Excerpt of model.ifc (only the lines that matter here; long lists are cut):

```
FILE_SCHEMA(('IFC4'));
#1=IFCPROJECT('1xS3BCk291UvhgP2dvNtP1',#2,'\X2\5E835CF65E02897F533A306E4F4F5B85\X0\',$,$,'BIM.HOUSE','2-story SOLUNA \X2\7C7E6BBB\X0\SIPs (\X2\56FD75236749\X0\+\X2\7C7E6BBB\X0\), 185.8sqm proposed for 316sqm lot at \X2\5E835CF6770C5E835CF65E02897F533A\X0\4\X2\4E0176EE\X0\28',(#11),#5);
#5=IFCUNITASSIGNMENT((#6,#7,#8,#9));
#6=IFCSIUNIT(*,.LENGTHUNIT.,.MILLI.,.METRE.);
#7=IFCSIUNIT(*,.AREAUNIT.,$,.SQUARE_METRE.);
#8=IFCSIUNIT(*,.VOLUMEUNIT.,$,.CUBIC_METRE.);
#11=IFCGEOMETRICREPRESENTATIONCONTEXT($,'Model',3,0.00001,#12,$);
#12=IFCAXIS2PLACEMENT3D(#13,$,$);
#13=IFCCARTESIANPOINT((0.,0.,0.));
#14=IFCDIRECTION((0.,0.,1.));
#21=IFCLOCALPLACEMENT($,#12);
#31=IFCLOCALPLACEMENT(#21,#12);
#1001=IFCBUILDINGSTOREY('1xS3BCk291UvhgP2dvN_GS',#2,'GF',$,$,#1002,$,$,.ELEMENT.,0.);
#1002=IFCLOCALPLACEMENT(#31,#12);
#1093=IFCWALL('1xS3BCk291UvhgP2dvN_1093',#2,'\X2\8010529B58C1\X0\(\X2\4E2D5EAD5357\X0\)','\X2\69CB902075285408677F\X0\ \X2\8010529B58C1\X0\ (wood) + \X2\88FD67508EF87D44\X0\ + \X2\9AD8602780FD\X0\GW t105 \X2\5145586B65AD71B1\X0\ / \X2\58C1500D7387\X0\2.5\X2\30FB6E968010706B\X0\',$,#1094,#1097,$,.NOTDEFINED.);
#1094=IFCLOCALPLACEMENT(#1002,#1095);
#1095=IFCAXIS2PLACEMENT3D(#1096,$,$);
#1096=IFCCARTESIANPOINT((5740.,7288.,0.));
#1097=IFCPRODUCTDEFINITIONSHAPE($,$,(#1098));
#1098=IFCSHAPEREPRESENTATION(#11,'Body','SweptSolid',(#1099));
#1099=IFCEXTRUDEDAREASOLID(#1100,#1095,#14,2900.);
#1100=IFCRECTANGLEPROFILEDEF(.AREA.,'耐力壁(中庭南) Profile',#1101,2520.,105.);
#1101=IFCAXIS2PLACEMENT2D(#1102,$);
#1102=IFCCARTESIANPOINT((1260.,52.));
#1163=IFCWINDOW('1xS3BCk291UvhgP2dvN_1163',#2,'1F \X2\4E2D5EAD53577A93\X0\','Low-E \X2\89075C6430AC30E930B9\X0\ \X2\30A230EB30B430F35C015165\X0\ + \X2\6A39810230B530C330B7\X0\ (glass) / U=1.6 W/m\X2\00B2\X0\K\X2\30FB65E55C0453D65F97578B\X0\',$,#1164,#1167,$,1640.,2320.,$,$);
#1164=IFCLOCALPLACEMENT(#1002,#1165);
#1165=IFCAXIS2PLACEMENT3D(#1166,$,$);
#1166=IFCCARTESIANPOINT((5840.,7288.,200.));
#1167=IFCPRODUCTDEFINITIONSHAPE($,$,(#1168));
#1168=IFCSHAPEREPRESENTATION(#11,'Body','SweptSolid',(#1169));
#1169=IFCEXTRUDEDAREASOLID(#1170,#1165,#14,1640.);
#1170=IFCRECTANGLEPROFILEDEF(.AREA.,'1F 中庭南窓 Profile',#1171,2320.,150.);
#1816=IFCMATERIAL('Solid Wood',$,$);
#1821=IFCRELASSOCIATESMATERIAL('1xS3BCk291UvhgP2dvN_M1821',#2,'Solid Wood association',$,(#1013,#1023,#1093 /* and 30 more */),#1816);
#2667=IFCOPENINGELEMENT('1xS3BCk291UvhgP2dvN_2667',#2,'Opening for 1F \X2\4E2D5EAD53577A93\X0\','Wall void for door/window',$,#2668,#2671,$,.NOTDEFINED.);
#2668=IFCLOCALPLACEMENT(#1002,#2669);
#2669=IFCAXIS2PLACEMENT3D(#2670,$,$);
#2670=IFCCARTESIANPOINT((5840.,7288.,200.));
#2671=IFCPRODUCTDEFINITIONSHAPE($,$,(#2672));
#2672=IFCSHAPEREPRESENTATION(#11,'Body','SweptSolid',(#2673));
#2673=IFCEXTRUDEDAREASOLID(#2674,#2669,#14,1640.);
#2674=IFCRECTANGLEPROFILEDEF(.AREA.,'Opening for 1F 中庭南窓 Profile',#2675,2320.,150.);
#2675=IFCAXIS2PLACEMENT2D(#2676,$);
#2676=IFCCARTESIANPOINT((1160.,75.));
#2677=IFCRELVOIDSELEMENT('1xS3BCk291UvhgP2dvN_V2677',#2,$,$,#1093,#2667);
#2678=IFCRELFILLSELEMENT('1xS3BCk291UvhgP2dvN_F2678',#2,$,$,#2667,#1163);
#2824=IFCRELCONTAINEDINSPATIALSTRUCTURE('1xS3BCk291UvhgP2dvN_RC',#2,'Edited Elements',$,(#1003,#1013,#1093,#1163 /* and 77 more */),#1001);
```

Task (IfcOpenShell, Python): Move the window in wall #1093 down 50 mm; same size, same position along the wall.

```python
import numpy as np
import ifcopenshell
import ifcopenshell.api.geometry
import ifcopenshell.util.placement
import ifcopenshell.util.unit

model = ifcopenshell.open("model.ifc")
unit_scale = ifcopenshell.util.unit.calculate_unit_scale(model)

window = model.by_guid("1xS3BCk291UvhgP2dvN_1163")
opening = window.FillsVoids[0].RelatingOpeningElement
dz = -0.05 / unit_scale

shift = np.array([0.0, 0.0, dz])
# The window is not placed relative to its opening, so move both.
for product in (opening, window):
    matrix = ifcopenshell.util.placement.get_local_placement(product.ObjectPlacement)
    matrix[:3, 3] += shift
    ifcopenshell.api.geometry.edit_object_placement(model, product=product, matrix=matrix, is_si=False)

print(f"moved by {dz * unit_scale:+.3f} m")

model.write("model-out.ifc")
```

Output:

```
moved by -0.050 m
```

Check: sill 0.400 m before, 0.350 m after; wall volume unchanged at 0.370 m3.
